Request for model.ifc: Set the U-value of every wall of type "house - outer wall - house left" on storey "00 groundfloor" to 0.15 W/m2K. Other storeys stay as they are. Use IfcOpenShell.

First a look at what the model holds.

```python
import ifcopenshell
import ifcopenshell.util.element

model = ifcopenshell.open("model.ifc")
print(model.schema)
storey = next(s for s in model.by_type("IfcBuildingStorey") if s.Name == "00 groundfloor")
walls = [e for e in ifcopenshell.util.element.get_decomposition(storey) if e.is_a("IfcWall")]
seen = {}
for e in walls:
    element_type = ifcopenshell.util.element.get_type(e)
    key = (element_type.Name if element_type != e and element_type else None, ifcopenshell.util.element.get_pset(e, "Pset_WallCommon", "ThermalTransmittance"))
    seen[key] = seen.get(key, 0) + 1
for (name, value), count in sorted(seen.items(), key=str):
    print(count, "x", name, "|", value)
```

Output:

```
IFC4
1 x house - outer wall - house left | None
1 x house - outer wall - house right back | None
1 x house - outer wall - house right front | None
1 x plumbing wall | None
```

```python
import ifcopenshell
import ifcopenshell.api.pset
import ifcopenshell.util.element

model = ifcopenshell.open("model.ifc")

storey = next(s for s in model.by_type("IfcBuildingStorey") if s.Name == "00 groundfloor")
walls = [e for e in ifcopenshell.util.element.get_decomposition(storey) if e.is_a("IfcWall")]

count = 0
for e in walls:
    element_type = ifcopenshell.util.element.get_type(e)
    if element_type in (None, e) or element_type.Name != "house - outer wall - house left":
        continue
    # add_pset returns the element's existing set when there is one.
    pset = ifcopenshell.api.pset.add_pset(model, product=e, name="Pset_WallCommon")
    ifcopenshell.api.pset.edit_pset(model, pset=pset, properties={"ThermalTransmittance": 0.15})
    count += 1

print(count, "walls updated")

model.write("model-out.ifc")
```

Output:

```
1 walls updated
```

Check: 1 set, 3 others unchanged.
